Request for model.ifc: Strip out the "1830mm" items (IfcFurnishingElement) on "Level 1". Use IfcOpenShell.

First a look at what the model holds.

```python
import ifcopenshell
import ifcopenshell.util.element

model = ifcopenshell.open("model.ifc")
print(model.schema)
storey = next(s for s in model.by_type("IfcBuildingStorey") if s.Name == "Level 1")
furniture = [e for e in ifcopenshell.util.element.get_decomposition(storey) if e.is_a("IfcFurnishingElement")]
seen = {}
for e in furniture:
    element_type = ifcopenshell.util.element.get_type(e)
    name = element_type.Name if element_type not in (None, e) else None
    seen[name] = seen.get(name, 0) + 1
for name, count in sorted(seen.items(), key=str):
    print(count, "x", name)
```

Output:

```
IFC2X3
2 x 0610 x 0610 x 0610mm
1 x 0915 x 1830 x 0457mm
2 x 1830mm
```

```python
import ifcopenshell
import ifcopenshell.api.root
import ifcopenshell.util.element

model = ifcopenshell.open("model.ifc")

storey = next(s for s in model.by_type("IfcBuildingStorey") if s.Name == "Level 1")
furniture = [e for e in ifcopenshell.util.element.get_decomposition(storey) if e.is_a("IfcFurnishingElement")]
targets = [e for e in furniture if (t := ifcopenshell.util.element.get_type(e)) not in (None, e) and t.Name == "1830mm"]

for e in targets:
    ifcopenshell.api.root.remove_product(model, product=e)
print(len(targets), "removed")

model.write("model_rev.ifc")
```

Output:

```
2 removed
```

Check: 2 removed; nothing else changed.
